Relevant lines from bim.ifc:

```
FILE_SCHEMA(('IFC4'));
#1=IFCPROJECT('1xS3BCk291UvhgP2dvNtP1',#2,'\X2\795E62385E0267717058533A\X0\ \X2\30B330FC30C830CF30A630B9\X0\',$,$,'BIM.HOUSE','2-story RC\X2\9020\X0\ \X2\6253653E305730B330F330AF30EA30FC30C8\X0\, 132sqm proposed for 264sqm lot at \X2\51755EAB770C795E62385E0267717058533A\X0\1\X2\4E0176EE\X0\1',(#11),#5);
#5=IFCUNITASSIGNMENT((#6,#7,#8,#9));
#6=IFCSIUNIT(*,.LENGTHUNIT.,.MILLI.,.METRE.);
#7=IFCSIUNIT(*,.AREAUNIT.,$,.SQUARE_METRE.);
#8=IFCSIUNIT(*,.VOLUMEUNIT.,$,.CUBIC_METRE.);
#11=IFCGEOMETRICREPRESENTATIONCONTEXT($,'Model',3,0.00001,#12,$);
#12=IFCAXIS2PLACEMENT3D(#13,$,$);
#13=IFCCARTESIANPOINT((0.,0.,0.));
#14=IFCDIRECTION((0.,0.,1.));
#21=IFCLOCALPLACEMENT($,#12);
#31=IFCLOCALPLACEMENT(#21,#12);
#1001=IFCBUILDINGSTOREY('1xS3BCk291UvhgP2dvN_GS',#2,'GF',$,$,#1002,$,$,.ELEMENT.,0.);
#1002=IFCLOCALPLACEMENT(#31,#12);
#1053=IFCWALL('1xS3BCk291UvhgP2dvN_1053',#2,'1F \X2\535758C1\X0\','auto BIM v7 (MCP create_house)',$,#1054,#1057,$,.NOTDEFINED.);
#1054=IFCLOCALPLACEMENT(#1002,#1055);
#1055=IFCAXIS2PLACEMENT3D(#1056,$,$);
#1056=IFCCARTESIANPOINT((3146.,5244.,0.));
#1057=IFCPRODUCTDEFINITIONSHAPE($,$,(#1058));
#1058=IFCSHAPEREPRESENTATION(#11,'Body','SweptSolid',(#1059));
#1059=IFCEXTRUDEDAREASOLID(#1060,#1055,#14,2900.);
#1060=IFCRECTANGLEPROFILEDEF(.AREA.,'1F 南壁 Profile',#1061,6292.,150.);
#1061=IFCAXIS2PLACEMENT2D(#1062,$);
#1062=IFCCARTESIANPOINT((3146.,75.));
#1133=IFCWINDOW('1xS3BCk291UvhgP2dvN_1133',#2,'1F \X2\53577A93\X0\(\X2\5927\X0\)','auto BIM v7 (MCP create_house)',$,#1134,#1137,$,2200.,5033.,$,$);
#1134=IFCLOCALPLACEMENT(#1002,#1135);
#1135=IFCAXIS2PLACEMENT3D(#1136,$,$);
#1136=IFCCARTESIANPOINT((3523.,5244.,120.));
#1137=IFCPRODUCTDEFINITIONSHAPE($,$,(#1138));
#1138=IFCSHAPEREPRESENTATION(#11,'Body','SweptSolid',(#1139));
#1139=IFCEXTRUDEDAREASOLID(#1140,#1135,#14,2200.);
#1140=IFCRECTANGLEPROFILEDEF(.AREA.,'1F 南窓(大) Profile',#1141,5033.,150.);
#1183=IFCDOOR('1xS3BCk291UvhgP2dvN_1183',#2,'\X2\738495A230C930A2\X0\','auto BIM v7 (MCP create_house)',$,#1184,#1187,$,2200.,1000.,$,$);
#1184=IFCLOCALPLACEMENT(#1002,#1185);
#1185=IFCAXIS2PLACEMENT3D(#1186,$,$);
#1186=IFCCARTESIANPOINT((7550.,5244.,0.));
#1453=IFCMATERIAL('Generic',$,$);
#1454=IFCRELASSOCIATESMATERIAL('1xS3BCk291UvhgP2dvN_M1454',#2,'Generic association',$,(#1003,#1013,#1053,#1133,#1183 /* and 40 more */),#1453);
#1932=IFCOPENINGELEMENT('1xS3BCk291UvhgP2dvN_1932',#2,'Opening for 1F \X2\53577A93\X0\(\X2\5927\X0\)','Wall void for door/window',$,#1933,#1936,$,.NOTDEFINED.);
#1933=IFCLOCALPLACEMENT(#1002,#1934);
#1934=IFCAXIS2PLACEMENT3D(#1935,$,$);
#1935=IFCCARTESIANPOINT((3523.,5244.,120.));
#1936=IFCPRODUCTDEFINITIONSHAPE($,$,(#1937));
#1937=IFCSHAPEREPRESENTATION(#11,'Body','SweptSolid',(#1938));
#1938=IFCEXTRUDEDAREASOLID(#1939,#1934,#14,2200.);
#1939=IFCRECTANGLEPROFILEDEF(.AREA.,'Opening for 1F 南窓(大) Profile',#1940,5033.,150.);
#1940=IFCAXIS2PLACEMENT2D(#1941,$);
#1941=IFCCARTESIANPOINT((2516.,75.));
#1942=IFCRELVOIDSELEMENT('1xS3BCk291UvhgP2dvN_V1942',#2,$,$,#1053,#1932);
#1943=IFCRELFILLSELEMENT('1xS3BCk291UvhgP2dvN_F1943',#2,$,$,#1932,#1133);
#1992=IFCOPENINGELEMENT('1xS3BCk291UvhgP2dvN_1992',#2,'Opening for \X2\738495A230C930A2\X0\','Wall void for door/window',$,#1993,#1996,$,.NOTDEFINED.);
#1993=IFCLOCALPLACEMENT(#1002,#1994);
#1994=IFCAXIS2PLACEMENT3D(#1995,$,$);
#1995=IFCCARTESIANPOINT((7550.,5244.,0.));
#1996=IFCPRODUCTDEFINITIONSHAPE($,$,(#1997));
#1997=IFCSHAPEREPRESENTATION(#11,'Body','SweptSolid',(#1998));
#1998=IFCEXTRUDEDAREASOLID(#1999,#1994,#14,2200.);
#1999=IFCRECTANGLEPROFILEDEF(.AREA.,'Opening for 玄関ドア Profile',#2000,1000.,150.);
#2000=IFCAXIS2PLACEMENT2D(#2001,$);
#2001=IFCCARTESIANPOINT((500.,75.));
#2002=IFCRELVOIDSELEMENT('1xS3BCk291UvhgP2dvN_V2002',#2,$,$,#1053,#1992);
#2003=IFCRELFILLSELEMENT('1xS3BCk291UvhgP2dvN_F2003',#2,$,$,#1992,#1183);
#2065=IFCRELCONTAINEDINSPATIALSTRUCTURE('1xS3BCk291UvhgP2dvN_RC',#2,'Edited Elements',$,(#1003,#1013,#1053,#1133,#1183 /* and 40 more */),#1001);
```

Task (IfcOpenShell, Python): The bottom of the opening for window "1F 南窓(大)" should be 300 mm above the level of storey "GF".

```python
import numpy as np
import ifcopenshell
import ifcopenshell.api.geometry
import ifcopenshell.geom
import ifcopenshell.util.element
import ifcopenshell.util.placement
import ifcopenshell.util.shape
import ifcopenshell.util.unit

model = ifcopenshell.open("bim.ifc")
unit_scale = ifcopenshell.util.unit.calculate_unit_scale(model)

window = model.by_id(1133)
opening = window.FillsVoids[0].RelatingOpeningElement
storey = ifcopenshell.util.element.get_container(window, ifc_class="IfcBuildingStorey")
level = ifcopenshell.util.placement.get_local_placement(storey.ObjectPlacement)[2, 3]

# The opening's origin need not be at the sill, so measure its lowest point.
shape = ifcopenshell.geom.create_shape(ifcopenshell.geom.settings(), opening)
bottom = ifcopenshell.util.shape.get_shape_bottom_elevation(shape, shape.geometry) / unit_scale
dz = level + 300.0 - bottom

shift = np.array([0.0, 0.0, dz])
# The window is not placed relative to its opening, so move both.
for product in (opening, window):
    matrix = ifcopenshell.util.placement.get_local_placement(product.ObjectPlacement)
    matrix[:3, 3] += shift
    ifcopenshell.api.geometry.edit_object_placement(model, product=product, matrix=matrix, is_si=False)

print(f"moved by {dz * unit_scale:+.3f} m")

model.write("bim_edited.ifc")
```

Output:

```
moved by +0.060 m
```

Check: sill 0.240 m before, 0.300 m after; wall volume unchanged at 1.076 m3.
